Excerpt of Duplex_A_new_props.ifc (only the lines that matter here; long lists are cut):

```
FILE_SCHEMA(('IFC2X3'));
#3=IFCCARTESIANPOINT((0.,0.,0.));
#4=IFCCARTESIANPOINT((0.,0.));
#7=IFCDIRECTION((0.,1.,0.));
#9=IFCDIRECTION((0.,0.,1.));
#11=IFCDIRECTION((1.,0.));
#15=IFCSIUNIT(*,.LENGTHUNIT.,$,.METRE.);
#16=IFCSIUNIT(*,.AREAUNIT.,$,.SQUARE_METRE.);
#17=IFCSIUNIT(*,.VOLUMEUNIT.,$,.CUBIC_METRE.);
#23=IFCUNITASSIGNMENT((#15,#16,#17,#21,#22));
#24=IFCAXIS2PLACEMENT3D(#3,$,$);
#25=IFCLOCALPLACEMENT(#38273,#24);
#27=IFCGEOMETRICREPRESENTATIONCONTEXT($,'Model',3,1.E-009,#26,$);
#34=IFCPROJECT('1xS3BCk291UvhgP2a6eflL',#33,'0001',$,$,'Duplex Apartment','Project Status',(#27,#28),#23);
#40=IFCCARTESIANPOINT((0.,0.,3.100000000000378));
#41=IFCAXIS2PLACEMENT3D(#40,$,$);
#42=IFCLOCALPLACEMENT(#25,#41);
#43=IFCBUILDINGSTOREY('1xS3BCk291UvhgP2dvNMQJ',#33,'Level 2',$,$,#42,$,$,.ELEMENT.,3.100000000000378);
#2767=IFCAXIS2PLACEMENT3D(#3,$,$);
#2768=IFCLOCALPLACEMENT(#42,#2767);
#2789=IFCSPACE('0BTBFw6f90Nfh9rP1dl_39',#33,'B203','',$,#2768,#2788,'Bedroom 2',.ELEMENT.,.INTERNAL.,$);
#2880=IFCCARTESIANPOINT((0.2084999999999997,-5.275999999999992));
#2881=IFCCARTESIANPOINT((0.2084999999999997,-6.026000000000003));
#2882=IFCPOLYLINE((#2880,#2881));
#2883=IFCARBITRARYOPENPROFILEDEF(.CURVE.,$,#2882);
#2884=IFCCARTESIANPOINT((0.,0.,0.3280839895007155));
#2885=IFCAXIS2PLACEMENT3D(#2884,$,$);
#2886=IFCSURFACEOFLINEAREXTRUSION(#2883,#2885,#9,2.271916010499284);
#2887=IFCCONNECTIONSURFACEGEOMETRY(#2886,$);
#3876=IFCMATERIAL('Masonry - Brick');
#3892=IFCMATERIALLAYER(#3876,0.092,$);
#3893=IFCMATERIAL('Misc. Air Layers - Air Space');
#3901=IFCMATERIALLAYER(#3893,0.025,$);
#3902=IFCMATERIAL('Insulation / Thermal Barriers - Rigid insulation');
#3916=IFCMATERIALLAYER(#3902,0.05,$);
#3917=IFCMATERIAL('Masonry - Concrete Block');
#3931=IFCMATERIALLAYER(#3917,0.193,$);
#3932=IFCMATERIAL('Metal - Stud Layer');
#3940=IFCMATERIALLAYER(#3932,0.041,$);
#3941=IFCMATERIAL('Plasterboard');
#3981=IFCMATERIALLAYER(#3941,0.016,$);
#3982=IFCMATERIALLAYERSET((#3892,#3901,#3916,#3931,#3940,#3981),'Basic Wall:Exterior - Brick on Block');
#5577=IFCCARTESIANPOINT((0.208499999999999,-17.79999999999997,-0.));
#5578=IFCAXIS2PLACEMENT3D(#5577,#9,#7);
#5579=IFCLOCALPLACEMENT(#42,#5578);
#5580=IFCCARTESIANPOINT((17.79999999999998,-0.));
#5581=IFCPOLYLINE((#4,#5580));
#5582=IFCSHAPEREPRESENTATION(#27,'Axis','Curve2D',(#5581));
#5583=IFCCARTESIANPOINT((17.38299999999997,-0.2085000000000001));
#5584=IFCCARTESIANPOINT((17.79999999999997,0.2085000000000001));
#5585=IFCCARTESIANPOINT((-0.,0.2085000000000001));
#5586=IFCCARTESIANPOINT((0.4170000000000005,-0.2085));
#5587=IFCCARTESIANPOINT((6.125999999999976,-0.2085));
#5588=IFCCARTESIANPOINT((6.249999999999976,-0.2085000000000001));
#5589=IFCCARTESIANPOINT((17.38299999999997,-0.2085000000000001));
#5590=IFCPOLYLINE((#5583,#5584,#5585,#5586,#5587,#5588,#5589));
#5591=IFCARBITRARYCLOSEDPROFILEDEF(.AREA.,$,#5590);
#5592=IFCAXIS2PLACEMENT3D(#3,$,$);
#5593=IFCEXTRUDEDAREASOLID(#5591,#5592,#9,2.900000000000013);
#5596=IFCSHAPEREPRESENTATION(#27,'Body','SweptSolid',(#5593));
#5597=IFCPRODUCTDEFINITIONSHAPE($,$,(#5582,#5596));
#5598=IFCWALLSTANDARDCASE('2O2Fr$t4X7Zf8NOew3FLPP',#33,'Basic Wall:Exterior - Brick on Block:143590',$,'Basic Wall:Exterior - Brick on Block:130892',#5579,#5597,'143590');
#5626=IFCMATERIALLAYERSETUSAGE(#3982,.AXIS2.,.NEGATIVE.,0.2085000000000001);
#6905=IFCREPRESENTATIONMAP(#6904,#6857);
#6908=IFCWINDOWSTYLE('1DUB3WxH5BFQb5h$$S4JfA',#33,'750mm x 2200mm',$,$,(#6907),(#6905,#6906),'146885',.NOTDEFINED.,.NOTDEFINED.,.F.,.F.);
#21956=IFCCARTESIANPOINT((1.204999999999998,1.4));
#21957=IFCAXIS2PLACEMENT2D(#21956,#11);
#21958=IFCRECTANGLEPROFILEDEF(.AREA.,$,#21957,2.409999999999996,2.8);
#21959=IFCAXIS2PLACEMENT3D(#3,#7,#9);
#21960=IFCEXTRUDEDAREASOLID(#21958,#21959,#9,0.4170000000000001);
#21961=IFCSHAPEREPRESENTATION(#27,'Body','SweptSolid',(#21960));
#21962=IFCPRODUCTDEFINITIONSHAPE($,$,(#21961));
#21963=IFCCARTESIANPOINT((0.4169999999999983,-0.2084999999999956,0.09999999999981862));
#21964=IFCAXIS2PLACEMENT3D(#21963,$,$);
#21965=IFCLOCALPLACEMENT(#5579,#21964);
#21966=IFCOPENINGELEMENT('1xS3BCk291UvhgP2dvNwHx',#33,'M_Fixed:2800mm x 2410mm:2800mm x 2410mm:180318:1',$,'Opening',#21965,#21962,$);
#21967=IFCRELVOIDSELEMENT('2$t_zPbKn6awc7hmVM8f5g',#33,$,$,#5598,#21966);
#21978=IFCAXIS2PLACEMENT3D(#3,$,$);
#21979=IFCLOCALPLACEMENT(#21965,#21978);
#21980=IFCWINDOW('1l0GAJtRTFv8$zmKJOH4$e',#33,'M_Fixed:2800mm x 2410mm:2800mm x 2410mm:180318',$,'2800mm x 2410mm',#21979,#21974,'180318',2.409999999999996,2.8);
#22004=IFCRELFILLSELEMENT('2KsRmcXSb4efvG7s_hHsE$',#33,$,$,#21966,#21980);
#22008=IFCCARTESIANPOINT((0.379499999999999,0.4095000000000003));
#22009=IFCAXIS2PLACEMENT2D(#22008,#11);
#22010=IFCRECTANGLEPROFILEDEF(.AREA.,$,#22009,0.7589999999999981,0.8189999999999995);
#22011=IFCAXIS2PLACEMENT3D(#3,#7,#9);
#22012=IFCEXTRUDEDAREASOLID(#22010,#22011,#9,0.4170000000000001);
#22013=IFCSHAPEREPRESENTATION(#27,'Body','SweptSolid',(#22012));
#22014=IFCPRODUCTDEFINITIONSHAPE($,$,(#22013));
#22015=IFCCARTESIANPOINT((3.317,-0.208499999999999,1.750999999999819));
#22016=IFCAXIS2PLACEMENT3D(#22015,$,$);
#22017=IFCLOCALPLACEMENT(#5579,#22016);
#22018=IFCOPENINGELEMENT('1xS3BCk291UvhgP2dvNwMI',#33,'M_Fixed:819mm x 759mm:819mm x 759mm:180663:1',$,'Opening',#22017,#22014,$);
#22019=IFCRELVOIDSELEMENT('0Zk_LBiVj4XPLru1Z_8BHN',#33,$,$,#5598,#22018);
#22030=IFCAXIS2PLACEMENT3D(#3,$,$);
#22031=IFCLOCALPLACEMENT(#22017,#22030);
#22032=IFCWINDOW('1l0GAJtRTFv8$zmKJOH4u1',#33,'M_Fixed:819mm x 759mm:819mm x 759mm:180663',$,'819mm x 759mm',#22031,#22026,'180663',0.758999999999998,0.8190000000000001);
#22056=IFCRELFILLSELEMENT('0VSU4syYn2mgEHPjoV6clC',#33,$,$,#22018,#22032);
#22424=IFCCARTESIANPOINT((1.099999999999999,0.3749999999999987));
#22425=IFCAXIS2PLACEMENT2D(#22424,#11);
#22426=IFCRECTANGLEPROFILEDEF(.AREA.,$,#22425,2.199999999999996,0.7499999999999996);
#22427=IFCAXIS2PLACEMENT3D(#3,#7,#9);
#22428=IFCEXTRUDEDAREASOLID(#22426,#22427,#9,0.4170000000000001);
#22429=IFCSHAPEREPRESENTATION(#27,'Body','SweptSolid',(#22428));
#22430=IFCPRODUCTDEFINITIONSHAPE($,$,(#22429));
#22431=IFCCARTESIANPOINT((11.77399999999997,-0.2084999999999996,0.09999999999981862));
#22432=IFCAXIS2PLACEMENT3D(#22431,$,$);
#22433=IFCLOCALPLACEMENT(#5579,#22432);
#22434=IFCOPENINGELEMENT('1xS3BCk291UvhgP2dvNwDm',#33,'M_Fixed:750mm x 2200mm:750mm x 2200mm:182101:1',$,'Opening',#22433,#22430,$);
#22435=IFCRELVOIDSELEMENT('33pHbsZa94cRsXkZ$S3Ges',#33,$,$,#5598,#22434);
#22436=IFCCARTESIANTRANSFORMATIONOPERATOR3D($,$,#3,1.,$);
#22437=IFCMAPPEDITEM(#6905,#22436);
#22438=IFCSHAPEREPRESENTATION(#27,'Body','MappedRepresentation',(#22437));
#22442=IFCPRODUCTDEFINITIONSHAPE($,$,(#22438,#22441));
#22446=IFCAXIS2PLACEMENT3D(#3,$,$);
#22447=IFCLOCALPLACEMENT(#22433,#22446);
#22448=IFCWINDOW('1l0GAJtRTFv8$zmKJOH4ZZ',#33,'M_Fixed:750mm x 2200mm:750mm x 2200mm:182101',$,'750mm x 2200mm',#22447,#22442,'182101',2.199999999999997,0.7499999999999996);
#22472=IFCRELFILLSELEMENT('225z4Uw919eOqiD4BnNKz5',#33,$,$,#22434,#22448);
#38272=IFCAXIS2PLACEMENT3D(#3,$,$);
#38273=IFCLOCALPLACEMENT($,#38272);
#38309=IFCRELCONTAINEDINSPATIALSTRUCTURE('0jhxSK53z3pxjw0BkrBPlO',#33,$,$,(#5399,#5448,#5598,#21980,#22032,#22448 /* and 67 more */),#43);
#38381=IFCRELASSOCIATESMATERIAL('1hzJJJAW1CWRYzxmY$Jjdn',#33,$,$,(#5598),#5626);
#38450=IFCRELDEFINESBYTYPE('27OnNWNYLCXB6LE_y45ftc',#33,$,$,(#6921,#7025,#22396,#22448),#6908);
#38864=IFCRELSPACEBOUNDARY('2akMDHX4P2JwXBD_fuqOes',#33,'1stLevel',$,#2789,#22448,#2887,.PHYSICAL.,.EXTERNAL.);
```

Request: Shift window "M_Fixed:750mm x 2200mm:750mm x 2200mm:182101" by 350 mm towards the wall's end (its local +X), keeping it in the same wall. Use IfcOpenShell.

```python
import numpy as np
import ifcopenshell
import ifcopenshell.api.geometry
import ifcopenshell.util.placement

model = ifcopenshell.open("Duplex_A_new_props.ifc")

window = model.by_guid("1l0GAJtRTFv8$zmKJOH4ZZ")
opening = window.FillsVoids[0].RelatingOpeningElement
wall = opening.VoidsElements[0].RelatingBuildingElement

wall_matrix = ifcopenshell.util.placement.get_local_placement(wall.ObjectPlacement)
shift = wall_matrix[:3, 0] * 0.35
before = ifcopenshell.util.placement.get_local_placement(window.ObjectPlacement)[:3, 3].copy()

# The window is placed relative to its opening, so it follows when the opening moves.
matrix = ifcopenshell.util.placement.get_local_placement(opening.ObjectPlacement)
matrix[:3, 3] += shift
ifcopenshell.api.geometry.edit_object_placement(
    model, product=opening, matrix=matrix, is_si=False, should_transform_children=True
)

# Space boundary surfaces are stored in each space's coordinates; move them too.
for rel in window.ProvidesBoundaries:
    if not rel.ConnectionGeometry:
        continue
    surface = rel.ConnectionGeometry.SurfaceOnRelatingElement
    space_matrix = ifcopenshell.util.placement.get_local_placement(rel.RelatingSpace.ObjectPlacement)
    point = np.array(surface.Position.Location.Coordinates) + space_matrix[:3, :3].T @ shift
    surface.Position = model.createIfcAxis2Placement3D(
        model.createIfcCartesianPoint(point.tolist()), surface.Position.Axis, surface.Position.RefDirection
    )

after = ifcopenshell.util.placement.get_local_placement(window.ObjectPlacement)[:3, 3]
print("window moved by", (after - before).round(3) + 0.0)

model.write("Duplex_A_new_props_updated.ifc")
```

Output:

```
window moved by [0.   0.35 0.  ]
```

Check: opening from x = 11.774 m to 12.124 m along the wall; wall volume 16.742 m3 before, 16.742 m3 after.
